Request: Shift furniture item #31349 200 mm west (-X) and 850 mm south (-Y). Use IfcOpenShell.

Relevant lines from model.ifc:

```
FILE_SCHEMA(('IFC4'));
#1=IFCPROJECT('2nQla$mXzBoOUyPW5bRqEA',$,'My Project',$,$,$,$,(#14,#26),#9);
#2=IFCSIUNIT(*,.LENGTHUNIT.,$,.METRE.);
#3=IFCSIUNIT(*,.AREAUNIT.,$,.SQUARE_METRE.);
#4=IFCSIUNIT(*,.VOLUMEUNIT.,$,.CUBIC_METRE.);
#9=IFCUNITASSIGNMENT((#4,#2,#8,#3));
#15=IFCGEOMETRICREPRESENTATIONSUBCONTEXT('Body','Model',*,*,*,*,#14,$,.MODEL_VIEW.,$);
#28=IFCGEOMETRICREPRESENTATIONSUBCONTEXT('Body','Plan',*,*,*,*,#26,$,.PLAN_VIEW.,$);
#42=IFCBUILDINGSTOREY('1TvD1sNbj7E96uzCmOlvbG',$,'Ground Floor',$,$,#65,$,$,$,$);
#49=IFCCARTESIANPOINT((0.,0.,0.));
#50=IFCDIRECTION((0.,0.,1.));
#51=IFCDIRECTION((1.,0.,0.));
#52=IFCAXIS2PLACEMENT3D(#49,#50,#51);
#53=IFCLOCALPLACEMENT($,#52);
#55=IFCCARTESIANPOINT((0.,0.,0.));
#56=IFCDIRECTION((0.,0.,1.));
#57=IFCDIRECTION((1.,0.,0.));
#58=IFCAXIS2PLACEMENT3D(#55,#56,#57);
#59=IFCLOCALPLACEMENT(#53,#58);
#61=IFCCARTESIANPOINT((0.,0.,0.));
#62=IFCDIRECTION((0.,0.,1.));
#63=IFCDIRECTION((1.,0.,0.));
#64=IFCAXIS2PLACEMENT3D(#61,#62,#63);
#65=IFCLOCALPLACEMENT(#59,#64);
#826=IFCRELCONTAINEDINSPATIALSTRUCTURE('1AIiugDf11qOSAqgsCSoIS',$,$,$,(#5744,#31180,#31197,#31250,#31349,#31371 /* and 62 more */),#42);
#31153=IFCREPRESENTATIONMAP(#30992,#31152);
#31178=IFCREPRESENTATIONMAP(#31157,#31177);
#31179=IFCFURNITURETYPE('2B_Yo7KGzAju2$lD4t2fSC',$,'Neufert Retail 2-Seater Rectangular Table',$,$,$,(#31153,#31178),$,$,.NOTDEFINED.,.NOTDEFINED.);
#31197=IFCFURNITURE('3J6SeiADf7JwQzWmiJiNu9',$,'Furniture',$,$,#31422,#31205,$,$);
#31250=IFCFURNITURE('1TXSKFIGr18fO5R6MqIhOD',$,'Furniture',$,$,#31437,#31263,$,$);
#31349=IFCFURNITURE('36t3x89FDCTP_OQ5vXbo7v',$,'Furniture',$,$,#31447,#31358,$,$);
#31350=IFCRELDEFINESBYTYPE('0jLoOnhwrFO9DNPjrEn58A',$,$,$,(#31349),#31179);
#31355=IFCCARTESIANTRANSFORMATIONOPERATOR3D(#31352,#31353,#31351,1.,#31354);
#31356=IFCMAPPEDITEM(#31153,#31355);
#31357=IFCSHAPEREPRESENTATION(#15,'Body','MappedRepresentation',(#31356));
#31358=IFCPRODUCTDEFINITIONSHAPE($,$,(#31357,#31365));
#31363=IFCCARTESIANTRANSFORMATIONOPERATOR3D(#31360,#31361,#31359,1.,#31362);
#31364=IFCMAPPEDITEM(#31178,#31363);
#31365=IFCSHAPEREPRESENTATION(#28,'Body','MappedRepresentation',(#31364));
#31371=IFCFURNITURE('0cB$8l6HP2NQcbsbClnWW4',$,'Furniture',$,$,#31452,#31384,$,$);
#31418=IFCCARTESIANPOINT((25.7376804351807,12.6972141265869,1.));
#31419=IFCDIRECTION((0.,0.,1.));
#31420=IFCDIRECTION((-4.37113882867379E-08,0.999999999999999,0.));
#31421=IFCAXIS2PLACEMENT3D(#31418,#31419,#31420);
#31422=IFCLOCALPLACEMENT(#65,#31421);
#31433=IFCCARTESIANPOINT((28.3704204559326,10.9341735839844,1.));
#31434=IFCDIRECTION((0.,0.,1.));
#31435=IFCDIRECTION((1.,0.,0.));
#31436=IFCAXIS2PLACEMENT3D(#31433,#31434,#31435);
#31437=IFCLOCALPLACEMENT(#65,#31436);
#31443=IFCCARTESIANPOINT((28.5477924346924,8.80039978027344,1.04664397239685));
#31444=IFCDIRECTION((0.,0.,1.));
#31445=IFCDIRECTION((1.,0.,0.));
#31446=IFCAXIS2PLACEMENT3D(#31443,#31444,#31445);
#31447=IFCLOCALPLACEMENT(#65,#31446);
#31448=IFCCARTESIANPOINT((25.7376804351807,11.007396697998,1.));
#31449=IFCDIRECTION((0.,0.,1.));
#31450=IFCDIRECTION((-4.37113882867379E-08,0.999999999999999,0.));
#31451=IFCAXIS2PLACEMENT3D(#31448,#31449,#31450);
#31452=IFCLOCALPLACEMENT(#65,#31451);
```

```python
import ifcopenshell
import ifcopenshell.api.geometry
import ifcopenshell.util.placement
import ifcopenshell.util.unit

model = ifcopenshell.open("model.ifc")
unit_scale = ifcopenshell.util.unit.calculate_unit_scale(model)

item = model.by_id(31349)
matrix = ifcopenshell.util.placement.get_local_placement(item.ObjectPlacement)
matrix[0, 3] -= 0.2 / unit_scale
matrix[1, 3] -= 0.85 / unit_scale
ifcopenshell.api.geometry.edit_object_placement(model, product=item, matrix=matrix, is_si=False)

print(ifcopenshell.util.placement.get_local_placement(item.ObjectPlacement).round(3) + 0.0)

model.write("model_edited.ifc")
```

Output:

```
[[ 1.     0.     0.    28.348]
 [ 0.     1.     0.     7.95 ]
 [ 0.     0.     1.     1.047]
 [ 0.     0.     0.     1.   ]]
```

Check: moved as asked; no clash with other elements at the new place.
